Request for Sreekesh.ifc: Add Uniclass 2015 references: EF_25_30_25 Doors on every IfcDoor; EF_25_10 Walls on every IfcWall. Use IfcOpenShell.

First a look at what the model holds.

```python
import ifcopenshell

model = ifcopenshell.open("Sreekesh.ifc")
print(model.schema)
print("classifications:", [c.Name for c in model.by_type("IfcClassification")])
for ifc_class in ("IfcDoor", "IfcRoof", "IfcStair", "IfcWall", "IfcWindow"):
    print(ifc_class, len(model.by_type(ifc_class)))
```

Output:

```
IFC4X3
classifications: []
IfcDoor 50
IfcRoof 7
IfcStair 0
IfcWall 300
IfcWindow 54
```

```python
import ifcopenshell
import ifcopenshell.api.classification

model = ifcopenshell.open("Sreekesh.ifc")

system = ifcopenshell.api.classification.add_classification(model, classification="Uniclass 2015")

codes = {
    "IfcDoor": ("EF_25_30_25", "Doors"),
    "IfcWall": ("EF_25_10", "Walls"),
}
for ifc_class, (code, name) in codes.items():
    products = model.by_type(ifc_class)
    ifcopenshell.api.classification.add_reference(
        model, products=products, classification=system, identification=code, name=name
    )
    print(code, len(products))

model.write("Sreekesh-out.ifc")
```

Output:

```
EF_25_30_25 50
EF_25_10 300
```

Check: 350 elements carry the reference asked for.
